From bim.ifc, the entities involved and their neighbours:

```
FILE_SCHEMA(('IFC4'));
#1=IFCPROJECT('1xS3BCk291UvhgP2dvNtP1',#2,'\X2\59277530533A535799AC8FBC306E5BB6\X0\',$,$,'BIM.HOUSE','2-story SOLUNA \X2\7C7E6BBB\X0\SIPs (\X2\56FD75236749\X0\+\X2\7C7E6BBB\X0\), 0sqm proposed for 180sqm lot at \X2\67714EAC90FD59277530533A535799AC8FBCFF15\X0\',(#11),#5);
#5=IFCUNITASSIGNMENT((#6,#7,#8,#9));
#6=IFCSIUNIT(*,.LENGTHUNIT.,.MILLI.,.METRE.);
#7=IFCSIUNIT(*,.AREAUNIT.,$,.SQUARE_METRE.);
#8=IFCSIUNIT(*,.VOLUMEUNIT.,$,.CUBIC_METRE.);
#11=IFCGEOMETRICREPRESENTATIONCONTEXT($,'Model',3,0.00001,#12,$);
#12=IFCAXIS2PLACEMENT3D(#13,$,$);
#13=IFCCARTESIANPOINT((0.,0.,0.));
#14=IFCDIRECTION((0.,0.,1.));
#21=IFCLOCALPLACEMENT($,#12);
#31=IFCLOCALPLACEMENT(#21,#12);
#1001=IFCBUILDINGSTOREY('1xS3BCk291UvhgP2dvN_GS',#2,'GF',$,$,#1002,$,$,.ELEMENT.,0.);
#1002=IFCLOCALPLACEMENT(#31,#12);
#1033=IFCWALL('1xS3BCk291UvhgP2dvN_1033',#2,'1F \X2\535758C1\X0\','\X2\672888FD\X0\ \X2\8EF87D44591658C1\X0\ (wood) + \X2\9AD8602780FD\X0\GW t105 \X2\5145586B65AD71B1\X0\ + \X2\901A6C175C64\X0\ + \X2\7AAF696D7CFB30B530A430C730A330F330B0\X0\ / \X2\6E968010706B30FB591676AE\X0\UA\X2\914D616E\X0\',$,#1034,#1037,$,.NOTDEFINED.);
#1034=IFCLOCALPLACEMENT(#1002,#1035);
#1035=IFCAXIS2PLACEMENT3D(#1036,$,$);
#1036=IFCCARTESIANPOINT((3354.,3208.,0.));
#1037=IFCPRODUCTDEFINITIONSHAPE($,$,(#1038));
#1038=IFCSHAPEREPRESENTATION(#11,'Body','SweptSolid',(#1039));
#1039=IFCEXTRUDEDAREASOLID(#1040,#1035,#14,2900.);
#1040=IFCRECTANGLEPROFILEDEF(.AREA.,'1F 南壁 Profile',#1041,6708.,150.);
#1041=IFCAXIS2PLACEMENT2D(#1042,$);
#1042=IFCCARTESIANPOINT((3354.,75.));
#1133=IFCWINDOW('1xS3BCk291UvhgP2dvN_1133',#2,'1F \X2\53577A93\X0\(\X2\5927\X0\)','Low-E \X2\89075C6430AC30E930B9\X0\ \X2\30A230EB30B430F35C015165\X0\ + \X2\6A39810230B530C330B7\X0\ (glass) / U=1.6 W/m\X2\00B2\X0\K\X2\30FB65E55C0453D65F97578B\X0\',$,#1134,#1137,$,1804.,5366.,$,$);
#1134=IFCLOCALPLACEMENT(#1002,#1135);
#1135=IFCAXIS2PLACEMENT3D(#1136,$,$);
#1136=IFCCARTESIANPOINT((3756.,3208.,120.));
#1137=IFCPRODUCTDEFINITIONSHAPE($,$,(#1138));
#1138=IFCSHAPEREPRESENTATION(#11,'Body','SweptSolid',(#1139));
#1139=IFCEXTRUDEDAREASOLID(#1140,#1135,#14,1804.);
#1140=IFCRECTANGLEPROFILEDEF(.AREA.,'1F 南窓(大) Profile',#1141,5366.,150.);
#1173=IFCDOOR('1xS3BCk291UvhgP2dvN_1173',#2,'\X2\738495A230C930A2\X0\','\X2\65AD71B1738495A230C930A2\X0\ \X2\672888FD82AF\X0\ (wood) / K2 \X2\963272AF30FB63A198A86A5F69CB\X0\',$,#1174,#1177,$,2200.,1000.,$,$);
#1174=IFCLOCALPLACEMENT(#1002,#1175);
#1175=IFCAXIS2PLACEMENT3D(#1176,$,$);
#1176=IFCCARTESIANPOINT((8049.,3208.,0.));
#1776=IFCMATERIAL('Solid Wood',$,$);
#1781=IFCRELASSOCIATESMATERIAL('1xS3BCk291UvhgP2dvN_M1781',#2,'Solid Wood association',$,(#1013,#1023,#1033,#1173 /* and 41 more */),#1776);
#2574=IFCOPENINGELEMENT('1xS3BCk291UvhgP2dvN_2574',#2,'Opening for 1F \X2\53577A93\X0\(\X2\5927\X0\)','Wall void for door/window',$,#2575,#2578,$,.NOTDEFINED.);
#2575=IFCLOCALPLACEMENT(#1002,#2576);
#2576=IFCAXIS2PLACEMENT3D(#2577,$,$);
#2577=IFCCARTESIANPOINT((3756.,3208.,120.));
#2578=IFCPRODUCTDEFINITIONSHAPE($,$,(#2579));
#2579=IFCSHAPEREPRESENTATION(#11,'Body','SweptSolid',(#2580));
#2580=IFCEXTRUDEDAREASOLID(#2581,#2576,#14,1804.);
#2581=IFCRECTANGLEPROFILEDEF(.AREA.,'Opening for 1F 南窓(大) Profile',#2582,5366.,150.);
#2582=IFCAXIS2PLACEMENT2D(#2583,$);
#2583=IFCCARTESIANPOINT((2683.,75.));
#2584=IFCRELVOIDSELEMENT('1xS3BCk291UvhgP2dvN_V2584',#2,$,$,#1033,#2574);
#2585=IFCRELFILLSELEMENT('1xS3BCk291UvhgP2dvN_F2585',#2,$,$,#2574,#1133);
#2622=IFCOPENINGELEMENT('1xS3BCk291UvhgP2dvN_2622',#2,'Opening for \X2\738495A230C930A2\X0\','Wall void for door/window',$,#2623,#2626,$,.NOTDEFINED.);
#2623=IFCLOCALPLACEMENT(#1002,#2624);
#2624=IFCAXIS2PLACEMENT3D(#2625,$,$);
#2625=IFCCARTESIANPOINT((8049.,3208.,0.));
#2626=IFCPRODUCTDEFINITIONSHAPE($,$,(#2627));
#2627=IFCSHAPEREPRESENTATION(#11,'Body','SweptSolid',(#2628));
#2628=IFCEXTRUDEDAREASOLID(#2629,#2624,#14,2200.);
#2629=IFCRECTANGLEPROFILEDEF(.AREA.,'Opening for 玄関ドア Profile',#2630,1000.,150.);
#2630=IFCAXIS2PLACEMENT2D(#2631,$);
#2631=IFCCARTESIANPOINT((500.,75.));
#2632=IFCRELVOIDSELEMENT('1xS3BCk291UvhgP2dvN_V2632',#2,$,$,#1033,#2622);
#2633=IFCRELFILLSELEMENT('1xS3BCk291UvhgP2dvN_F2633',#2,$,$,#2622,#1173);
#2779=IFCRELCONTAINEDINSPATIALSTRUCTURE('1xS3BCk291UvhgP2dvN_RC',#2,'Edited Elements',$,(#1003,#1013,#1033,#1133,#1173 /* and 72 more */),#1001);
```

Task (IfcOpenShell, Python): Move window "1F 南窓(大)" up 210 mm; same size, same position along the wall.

```python
import numpy as np
import ifcopenshell
import ifcopenshell.api.geometry
import ifcopenshell.util.placement
import ifcopenshell.util.unit

model = ifcopenshell.open("bim.ifc")
unit_scale = ifcopenshell.util.unit.calculate_unit_scale(model)

window = model.by_guid("1xS3BCk291UvhgP2dvN_1133")
opening = window.FillsVoids[0].RelatingOpeningElement
dz = 0.21 / unit_scale

shift = np.array([0.0, 0.0, dz])
# The window is not placed relative to its opening, so move both.
for product in (opening, window):
    matrix = ifcopenshell.util.placement.get_local_placement(product.ObjectPlacement)
    matrix[:3, 3] += shift
    ifcopenshell.api.geometry.edit_object_placement(model, product=product, matrix=matrix, is_si=False)

print(f"moved by {dz * unit_scale:+.3f} m")

model.write("bim_updated.ifc")
```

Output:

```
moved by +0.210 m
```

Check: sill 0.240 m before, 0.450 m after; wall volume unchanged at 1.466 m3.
